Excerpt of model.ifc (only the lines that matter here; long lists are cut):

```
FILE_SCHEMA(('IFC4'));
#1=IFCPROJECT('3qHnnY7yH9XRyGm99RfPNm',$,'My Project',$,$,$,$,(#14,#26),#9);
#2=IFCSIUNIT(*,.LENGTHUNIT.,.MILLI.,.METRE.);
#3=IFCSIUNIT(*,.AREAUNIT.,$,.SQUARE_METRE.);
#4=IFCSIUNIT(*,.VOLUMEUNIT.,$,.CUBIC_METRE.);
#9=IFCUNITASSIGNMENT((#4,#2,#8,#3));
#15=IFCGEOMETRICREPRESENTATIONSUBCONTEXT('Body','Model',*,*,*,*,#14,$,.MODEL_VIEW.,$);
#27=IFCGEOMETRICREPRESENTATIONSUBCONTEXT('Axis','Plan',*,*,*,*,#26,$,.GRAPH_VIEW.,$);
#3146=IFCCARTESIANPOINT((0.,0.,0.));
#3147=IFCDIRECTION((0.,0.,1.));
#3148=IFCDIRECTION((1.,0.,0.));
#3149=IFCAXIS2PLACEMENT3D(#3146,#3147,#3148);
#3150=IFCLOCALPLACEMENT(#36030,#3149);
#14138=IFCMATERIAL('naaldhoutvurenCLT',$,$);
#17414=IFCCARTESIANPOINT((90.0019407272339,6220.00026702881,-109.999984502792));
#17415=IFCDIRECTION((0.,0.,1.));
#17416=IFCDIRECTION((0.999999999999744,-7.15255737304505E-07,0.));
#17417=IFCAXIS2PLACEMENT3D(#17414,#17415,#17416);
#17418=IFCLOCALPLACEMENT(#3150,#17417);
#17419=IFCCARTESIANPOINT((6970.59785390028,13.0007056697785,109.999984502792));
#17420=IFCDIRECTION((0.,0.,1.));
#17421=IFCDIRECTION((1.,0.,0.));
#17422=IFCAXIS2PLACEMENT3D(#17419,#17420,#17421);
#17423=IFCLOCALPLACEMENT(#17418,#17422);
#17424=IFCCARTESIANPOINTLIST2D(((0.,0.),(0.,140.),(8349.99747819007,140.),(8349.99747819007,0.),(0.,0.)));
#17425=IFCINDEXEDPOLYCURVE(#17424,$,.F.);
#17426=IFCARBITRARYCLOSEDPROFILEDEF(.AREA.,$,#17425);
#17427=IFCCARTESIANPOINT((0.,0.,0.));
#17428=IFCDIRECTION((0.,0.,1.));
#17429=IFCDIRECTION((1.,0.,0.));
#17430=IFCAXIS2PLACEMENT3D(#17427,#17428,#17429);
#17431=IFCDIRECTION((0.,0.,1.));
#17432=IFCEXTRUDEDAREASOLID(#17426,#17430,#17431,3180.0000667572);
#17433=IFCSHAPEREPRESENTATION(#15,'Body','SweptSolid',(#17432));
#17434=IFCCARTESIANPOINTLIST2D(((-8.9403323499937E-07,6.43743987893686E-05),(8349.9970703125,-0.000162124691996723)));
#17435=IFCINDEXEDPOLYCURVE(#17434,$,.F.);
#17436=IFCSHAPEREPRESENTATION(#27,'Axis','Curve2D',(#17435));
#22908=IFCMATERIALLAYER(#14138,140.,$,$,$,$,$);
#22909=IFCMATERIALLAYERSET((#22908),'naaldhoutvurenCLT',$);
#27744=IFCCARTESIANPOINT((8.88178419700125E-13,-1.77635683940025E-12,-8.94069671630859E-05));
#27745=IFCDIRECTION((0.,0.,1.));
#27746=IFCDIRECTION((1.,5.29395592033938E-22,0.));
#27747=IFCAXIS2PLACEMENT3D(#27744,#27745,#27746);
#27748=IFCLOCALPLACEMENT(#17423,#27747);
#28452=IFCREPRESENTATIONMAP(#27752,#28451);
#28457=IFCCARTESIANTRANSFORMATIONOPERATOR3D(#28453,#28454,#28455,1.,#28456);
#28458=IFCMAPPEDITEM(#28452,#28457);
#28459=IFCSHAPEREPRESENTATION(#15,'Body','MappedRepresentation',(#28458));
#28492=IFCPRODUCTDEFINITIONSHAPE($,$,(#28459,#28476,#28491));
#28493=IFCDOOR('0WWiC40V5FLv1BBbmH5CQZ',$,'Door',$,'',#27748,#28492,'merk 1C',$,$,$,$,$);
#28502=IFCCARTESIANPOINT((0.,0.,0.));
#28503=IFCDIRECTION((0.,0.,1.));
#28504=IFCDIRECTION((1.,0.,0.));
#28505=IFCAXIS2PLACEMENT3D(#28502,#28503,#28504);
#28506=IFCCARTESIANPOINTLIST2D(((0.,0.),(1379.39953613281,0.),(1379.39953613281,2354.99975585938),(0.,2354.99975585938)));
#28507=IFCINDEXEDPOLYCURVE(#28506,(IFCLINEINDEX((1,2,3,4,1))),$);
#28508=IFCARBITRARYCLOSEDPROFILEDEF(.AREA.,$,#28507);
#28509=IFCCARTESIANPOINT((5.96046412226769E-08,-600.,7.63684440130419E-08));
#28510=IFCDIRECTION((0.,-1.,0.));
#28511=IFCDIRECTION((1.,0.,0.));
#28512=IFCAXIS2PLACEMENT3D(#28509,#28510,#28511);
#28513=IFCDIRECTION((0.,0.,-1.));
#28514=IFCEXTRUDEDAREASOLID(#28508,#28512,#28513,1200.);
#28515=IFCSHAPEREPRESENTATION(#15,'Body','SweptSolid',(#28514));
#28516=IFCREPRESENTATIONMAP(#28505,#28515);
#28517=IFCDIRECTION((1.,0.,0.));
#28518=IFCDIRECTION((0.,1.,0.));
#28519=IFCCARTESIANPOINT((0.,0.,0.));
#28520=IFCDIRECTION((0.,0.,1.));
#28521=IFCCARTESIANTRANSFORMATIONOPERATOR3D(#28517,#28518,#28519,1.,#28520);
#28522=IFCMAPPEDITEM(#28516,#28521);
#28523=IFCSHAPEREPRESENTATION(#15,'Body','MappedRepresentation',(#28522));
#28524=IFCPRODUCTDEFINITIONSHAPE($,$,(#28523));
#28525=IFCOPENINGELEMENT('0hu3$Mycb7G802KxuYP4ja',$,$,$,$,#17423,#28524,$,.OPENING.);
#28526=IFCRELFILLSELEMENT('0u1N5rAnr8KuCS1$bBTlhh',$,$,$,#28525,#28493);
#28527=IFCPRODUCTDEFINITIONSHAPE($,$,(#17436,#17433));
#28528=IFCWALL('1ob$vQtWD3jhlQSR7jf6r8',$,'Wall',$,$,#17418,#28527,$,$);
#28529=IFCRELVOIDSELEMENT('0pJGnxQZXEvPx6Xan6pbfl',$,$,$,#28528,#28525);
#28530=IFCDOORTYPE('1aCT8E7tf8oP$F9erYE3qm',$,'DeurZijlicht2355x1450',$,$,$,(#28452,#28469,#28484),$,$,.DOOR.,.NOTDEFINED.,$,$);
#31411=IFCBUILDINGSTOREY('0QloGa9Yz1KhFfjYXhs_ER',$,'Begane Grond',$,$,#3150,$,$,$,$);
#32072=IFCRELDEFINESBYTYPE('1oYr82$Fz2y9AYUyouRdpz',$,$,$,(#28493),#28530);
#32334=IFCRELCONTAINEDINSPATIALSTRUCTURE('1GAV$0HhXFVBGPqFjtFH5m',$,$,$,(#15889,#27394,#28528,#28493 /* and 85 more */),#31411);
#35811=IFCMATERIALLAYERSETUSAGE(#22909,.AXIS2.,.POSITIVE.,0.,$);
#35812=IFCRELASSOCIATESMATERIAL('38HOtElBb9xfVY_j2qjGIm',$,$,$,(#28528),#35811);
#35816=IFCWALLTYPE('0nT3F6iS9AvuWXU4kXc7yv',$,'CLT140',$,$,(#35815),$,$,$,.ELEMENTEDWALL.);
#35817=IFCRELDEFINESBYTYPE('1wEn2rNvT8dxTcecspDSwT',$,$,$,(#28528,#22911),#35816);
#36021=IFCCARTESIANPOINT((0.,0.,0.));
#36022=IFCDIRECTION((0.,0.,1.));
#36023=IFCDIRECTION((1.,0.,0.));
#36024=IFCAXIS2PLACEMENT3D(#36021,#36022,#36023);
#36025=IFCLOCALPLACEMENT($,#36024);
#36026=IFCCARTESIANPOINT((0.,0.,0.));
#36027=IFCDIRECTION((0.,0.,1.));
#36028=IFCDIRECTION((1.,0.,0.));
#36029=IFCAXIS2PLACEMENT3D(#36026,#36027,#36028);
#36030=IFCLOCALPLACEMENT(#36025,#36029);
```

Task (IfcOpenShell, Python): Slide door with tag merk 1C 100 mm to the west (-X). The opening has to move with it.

```python
import ifcopenshell
import ifcopenshell.api.geometry
import ifcopenshell.util.placement

model = ifcopenshell.open("model.ifc")

door = model.by_guid("0WWiC40V5FLv1BBbmH5CQZ")
opening = door.FillsVoids[0].RelatingOpeningElement
wall = opening.VoidsElements[0].RelatingBuildingElement

wall_matrix = ifcopenshell.util.placement.get_local_placement(wall.ObjectPlacement)
shift = wall_matrix[:3, 0] * -100.0
before = ifcopenshell.util.placement.get_local_placement(door.ObjectPlacement)[:3, 3].copy()

# The door is placed relative to its opening, so it follows when the opening moves.
matrix = ifcopenshell.util.placement.get_local_placement(opening.ObjectPlacement)
matrix[:3, 3] += shift
ifcopenshell.api.geometry.edit_object_placement(
    model, product=opening, matrix=matrix, is_si=False, should_transform_children=True
)

after = ifcopenshell.util.placement.get_local_placement(door.ObjectPlacement)[:3, 3]
print("door moved by", (after - before).round(3) + 0.0)

model.write("model_v2.ifc")
```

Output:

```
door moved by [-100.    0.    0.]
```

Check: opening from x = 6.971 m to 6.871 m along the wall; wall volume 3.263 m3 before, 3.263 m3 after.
